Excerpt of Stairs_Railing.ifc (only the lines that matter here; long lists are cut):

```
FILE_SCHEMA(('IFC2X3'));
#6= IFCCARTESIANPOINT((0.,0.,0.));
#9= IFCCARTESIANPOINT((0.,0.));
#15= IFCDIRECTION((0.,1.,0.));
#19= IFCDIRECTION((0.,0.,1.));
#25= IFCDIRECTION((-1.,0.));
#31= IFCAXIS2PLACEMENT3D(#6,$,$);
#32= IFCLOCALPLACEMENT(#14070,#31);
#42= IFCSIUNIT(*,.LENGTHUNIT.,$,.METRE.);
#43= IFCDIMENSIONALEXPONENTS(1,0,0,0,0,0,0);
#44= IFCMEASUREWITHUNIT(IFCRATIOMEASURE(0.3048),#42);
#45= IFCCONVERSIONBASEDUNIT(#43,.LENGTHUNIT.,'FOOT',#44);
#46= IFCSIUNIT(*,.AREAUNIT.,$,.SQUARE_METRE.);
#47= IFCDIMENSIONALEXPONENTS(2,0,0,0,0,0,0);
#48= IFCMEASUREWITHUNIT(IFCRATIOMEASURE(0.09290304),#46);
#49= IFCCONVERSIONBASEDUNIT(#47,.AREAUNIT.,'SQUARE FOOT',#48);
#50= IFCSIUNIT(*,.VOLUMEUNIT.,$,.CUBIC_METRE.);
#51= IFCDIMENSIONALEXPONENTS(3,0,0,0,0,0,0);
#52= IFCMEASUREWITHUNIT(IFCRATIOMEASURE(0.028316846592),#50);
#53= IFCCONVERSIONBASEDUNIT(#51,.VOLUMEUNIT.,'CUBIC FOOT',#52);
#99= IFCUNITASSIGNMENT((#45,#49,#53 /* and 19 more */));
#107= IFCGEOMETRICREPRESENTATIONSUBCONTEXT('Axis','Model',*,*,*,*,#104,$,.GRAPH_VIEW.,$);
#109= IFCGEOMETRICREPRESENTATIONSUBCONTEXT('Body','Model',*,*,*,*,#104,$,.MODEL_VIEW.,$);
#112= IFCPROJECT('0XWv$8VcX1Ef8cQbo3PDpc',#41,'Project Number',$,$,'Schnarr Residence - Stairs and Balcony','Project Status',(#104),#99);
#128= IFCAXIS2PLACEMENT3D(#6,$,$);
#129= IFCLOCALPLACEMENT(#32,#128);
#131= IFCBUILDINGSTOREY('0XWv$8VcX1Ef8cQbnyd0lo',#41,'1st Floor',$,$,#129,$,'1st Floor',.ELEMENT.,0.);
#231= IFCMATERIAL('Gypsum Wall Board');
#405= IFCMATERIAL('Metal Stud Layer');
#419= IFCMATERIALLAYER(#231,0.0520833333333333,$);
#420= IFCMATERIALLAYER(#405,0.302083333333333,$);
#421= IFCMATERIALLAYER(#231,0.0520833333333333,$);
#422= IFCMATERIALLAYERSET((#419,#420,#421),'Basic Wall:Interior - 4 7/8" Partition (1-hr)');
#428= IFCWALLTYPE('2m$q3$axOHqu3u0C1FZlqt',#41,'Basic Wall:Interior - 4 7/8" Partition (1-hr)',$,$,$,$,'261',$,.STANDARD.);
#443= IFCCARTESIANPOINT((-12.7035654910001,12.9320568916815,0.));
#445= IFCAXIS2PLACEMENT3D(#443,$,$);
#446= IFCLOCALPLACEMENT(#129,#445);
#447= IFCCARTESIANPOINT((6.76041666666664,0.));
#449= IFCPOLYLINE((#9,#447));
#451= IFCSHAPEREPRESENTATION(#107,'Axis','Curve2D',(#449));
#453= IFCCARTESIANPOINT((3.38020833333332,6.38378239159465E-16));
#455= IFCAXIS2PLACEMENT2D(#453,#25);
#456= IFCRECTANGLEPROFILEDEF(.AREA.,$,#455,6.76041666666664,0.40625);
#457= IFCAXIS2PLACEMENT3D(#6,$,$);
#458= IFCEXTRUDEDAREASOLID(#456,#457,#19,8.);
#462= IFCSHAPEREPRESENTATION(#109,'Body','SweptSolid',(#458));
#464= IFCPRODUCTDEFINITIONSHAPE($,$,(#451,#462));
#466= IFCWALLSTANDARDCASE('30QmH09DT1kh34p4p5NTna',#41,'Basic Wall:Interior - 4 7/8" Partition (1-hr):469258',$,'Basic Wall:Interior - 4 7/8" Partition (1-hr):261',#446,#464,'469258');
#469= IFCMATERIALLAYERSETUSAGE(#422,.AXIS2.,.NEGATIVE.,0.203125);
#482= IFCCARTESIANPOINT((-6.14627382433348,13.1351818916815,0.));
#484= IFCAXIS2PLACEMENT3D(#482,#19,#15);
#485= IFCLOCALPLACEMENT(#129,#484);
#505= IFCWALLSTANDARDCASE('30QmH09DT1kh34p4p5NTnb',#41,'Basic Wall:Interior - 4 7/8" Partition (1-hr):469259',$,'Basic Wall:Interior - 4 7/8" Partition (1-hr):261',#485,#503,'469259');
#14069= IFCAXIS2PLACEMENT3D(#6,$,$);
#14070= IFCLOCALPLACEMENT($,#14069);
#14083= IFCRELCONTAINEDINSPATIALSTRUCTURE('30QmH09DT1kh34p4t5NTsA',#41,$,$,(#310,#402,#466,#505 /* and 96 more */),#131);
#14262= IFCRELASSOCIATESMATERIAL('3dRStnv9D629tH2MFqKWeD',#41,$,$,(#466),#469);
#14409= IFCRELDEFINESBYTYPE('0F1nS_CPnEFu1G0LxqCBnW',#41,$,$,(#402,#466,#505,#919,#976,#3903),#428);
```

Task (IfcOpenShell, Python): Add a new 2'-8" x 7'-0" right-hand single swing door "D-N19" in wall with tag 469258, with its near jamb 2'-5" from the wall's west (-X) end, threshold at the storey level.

```python
import numpy as np
import ifcopenshell
import ifcopenshell.api.feature
import ifcopenshell.api.geometry
import ifcopenshell.api.root
import ifcopenshell.api.spatial
import ifcopenshell.api.type
import ifcopenshell.geom
import ifcopenshell.util.element
import ifcopenshell.util.placement
import ifcopenshell.util.representation
import ifcopenshell.util.shape
import ifcopenshell.util.unit

model = ifcopenshell.open("Stairs_Railing.ifc")
unit_scale = ifcopenshell.util.unit.calculate_unit_scale(model)
settings = ifcopenshell.geom.settings()


def volume(element):
    """Net volume in cubic metres, openings subtracted."""
    shape = ifcopenshell.geom.create_shape(settings, element)
    return ifcopenshell.util.shape.get_volume(shape.geometry)


wall = model.by_guid("30QmH09DT1kh34p4p5NTna")
storey = ifcopenshell.util.element.get_container(wall, ifc_class="IfcBuildingStorey")
context = ifcopenshell.util.representation.get_context(model, "Model", "Body", "MODEL_VIEW")
before = volume(wall)

width, height, from_end, sill = 0.8128, 2.1336, 0.7366, 0.0  # metres

# The wall runs along its own X axis, and the end named is its -X end.
wall_shape = ifcopenshell.geom.create_shape(settings, wall)
x, y, z = ifcopenshell.util.shape.get_vertices(wall_shape.geometry).T
start = x.min() + from_end
face, thickness = float(y.min()), float(y.max() - y.min())
wall_matrix = ifcopenshell.util.placement.get_local_placement(wall.ObjectPlacement)
level = ifcopenshell.util.placement.get_local_placement(storey.ObjectPlacement)[2, 3]


def in_wall(x, y):
    """Placement at x, y metres in the wall's axes, at sill height."""
    matrix = wall_matrix.copy()
    matrix[:, 3] = wall_matrix @ np.array([x / unit_scale, y / unit_scale, 0.0, 1.0])
    matrix[2, 3] = level + sill / unit_scale
    return matrix


# Opening: a box that overshoots both wall faces by 50 mm.
opening = ifcopenshell.api.root.create_entity(model, ifc_class="IfcOpeningElement")
box = ifcopenshell.api.geometry.add_wall_representation(
    model, context=context, length=width, height=height, thickness=thickness + 0.1
)
ifcopenshell.api.geometry.assign_representation(model, product=opening, representation=box)
ifcopenshell.api.geometry.edit_object_placement(model, product=opening, matrix=in_wall(start, face - 0.05), is_si=False)
ifcopenshell.api.feature.add_feature(model, feature=opening, element=wall)

door = ifcopenshell.api.root.create_entity(model, ifc_class="IfcDoor", name="D-N19")
door.OverallWidth, door.OverallHeight = width / unit_scale, height / unit_scale
body = ifcopenshell.api.geometry.add_door_representation(
    model,
    context=context,
    overall_width=door.OverallWidth,
    overall_height=door.OverallHeight,
    operation_type="SINGLE_SWING_RIGHT",
    lining_properties={"LiningDepth": thickness / unit_scale, "ThresholdDepth": thickness / unit_scale},
)
ifcopenshell.api.geometry.assign_representation(model, product=door, representation=body)
ifcopenshell.api.spatial.assign_container(model, products=[door], relating_structure=storey)
fills = ifcopenshell.api.feature.add_filling(model, opening=opening, element=door)
fills.OwnerHistory = door.OwnerHistory  # required in IFC2X3

# IFC2X3 keeps the operation on the door style.
style = ifcopenshell.api.root.create_entity(model, ifc_class="IfcDoorStyle", name="D-N19")
style.OperationType, style.ConstructionType = "SINGLE_SWING_RIGHT", "NOTDEFINED"
style.ParameterTakesPrecedence = style.Sizeable = False
ifcopenshell.api.type.assign_type(model, related_objects=[door], relating_type=style)

# The lining spans the wall, so the door starts at the wall face.
ifcopenshell.api.geometry.edit_object_placement(model, product=door, matrix=in_wall(start, face), is_si=False)

after = volume(wall)

print(f"wall volume {before:.3f} -> {after:.3f} m3")

model.write("Stairs_Railing_edited.ifc")
```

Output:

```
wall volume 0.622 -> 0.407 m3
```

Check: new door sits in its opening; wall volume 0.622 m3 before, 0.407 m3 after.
